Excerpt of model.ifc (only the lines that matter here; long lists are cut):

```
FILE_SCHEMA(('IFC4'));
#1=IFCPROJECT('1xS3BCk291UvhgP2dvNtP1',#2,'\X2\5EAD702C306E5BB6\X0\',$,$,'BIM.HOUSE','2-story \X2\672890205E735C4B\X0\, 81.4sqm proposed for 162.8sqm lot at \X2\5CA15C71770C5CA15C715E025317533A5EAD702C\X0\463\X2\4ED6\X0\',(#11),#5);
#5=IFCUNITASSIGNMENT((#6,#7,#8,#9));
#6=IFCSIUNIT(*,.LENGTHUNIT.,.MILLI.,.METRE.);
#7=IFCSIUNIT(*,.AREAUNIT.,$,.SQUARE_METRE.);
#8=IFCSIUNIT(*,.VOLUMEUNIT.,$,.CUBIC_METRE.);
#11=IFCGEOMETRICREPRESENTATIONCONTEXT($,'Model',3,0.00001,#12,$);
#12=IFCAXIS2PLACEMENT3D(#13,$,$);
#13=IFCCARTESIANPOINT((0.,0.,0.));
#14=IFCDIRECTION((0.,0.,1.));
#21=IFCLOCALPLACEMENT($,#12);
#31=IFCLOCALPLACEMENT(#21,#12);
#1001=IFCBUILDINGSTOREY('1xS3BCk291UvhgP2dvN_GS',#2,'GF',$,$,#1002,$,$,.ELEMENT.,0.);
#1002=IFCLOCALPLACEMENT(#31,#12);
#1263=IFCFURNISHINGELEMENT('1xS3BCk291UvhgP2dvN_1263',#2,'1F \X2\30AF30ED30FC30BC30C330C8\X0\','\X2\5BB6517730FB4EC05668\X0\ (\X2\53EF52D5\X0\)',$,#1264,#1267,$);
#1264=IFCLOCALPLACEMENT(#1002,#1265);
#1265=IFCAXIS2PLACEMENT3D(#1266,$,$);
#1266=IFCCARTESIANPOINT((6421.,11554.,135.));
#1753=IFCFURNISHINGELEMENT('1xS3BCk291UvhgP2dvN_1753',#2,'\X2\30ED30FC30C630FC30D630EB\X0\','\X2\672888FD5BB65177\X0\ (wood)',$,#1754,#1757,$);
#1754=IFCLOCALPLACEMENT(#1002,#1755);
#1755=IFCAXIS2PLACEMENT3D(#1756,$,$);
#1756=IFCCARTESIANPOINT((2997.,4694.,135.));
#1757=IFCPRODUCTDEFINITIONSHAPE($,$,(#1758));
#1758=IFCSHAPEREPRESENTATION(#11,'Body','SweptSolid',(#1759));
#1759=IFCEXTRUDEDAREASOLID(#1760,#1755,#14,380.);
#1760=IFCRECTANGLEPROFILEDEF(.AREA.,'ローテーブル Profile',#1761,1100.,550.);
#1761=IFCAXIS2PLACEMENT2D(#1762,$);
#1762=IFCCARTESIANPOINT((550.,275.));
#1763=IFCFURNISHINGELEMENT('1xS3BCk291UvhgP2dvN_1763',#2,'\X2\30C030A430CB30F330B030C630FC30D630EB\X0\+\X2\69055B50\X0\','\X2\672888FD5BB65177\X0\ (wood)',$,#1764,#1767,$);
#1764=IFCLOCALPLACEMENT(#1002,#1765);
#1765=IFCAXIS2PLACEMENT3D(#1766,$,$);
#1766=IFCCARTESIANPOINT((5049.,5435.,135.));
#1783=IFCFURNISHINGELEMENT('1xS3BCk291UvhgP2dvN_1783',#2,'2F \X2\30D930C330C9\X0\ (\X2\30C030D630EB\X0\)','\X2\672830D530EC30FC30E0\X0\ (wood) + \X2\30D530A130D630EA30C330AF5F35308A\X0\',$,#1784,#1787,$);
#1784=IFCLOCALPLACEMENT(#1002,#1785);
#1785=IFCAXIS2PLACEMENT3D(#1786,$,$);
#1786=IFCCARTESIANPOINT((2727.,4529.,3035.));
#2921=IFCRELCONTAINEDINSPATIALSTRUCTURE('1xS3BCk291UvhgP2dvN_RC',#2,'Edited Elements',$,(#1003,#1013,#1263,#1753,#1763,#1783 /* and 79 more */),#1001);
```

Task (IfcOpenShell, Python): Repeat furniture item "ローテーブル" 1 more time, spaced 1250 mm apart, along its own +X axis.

```python
import ifcopenshell
import ifcopenshell.api.geometry
import ifcopenshell.api.root
import ifcopenshell.util.element
import ifcopenshell.util.placement

model = ifcopenshell.open("model.ifc")


def reuse_history(source, copy):
    """copy_class also copies each property set's owner history, people and application; keep the originals."""
    for rel in copy.IsDefinedBy:
        if rel.is_a("IfcRelDefinesByProperties") and (history := rel.RelatingPropertyDefinition.OwnerHistory):
            rel.RelatingPropertyDefinition.OwnerHistory = source.OwnerHistory
            ifcopenshell.util.element.remove_deep2(model, history)


source = model.by_guid("1xS3BCk291UvhgP2dvN_1753")
base = ifcopenshell.util.placement.get_local_placement(source.ObjectPlacement)
step = base[:3, 0] * 1250.0

for i in range(1, 2):
    copy = ifcopenshell.api.root.copy_class(model, product=source)
    copy.Representation = ifcopenshell.util.element.copy_deep(
        model, source.Representation, exclude=["IfcGeometricRepresentationContext", "IfcRepresentationMap"]
    )
    reuse_history(source, copy)
    matrix = base.copy()
    matrix[:3, 3] += i * step
    print("added at", matrix[:3, 3].round(3) + 0.0)
    ifcopenshell.api.geometry.edit_object_placement(model, product=copy, matrix=matrix, is_si=False)

model.write("model_edited.ifc")
```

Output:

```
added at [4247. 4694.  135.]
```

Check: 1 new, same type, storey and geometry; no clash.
